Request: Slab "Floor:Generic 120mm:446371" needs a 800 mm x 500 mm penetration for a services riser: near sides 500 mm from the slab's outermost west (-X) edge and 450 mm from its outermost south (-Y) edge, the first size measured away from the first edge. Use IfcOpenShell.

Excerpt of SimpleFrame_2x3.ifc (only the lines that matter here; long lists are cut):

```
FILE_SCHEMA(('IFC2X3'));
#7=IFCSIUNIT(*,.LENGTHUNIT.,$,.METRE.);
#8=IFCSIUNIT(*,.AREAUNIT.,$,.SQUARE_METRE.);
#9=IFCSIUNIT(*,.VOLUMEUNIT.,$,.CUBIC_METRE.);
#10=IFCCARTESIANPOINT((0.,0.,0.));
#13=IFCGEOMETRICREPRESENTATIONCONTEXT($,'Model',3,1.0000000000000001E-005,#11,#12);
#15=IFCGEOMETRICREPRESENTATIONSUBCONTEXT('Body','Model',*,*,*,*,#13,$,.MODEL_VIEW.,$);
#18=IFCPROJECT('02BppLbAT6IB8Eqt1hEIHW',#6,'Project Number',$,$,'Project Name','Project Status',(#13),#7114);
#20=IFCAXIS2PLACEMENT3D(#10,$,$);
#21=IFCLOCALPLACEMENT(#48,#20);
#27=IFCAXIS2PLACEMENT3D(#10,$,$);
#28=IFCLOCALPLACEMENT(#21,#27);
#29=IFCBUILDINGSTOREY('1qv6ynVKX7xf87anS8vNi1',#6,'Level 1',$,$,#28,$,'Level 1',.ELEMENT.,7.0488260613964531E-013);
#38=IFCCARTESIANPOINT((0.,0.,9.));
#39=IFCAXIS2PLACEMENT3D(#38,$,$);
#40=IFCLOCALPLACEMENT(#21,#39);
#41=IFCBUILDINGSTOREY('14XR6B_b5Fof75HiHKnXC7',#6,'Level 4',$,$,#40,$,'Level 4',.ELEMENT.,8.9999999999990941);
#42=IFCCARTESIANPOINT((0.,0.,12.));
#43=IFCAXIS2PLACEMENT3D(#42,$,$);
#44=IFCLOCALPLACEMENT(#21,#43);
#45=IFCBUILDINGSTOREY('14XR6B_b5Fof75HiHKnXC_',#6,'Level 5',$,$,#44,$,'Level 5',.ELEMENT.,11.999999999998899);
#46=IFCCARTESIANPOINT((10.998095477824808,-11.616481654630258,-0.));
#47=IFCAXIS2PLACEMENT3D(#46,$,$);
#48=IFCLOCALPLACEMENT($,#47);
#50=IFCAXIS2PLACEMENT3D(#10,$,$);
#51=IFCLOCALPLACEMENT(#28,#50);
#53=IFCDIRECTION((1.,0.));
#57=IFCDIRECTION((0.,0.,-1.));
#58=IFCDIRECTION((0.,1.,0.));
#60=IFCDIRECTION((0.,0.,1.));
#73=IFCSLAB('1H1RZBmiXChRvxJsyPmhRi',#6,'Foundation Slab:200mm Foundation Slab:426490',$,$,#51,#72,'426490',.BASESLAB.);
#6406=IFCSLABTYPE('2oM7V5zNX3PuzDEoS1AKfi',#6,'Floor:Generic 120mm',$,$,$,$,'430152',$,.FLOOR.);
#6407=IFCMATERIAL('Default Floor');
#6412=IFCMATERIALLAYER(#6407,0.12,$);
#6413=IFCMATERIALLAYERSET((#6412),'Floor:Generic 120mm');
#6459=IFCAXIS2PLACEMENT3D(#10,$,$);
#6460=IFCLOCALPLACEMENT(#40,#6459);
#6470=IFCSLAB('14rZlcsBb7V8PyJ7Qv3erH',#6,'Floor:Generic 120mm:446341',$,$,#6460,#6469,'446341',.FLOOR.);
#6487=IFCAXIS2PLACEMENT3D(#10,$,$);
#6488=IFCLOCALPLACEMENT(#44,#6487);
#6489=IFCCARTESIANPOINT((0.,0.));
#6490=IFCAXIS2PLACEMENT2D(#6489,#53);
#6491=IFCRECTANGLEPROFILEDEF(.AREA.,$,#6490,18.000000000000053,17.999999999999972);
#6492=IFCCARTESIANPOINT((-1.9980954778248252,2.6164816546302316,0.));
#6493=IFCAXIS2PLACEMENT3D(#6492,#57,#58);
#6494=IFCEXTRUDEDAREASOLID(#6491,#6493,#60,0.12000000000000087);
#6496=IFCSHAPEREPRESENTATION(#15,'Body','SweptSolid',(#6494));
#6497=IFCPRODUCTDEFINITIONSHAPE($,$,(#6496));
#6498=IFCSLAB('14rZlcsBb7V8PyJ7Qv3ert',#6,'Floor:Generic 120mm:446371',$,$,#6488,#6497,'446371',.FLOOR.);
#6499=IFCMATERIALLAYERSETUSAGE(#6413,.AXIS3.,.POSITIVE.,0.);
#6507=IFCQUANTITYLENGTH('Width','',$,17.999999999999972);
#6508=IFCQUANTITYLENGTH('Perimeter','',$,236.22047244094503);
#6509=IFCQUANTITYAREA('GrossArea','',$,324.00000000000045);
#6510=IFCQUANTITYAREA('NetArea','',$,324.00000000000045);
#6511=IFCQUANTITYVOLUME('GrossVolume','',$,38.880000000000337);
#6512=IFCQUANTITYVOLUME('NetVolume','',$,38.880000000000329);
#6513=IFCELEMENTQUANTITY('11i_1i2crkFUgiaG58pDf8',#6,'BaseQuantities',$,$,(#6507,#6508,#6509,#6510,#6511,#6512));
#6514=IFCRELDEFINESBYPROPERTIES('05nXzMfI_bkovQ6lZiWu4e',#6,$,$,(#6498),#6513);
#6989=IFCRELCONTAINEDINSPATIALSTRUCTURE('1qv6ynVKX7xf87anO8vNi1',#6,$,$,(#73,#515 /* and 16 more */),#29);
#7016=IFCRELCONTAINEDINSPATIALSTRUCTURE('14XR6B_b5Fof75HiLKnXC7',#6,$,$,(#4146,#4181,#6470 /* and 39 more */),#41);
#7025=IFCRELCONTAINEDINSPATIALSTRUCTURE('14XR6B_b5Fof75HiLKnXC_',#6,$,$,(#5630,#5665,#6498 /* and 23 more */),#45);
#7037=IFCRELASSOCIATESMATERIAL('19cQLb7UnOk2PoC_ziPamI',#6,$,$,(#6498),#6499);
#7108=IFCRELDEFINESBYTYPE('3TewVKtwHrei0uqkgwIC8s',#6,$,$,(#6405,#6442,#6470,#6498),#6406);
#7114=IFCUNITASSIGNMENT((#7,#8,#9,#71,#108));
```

```python
import numpy as np
import ifcopenshell
import ifcopenshell.api.feature
import ifcopenshell.api.geometry
import ifcopenshell.api.pset
import ifcopenshell.api.root
import ifcopenshell.geom
import ifcopenshell.util.element
import ifcopenshell.util.placement
import ifcopenshell.util.representation
import ifcopenshell.util.shape
import ifcopenshell.util.unit

model = ifcopenshell.open("SimpleFrame_2x3.ifc")
unit_scale = ifcopenshell.util.unit.calculate_unit_scale(model)
area_scale = ifcopenshell.util.unit.calculate_unit_scale(model, "AREAUNIT")
volume_scale = ifcopenshell.util.unit.calculate_unit_scale(model, "VOLUMEUNIT")
settings = ifcopenshell.geom.settings()


def volume(element):
    """Net volume in cubic metres, openings subtracted."""
    shape = ifcopenshell.geom.create_shape(settings, element)
    return ifcopenshell.util.shape.get_volume(shape.geometry)


slab = model.by_id(6498)
before = volume(slab)

# Extent in the slab's own axes, in metres. The edges named are its -X and -Y sides.
slab_shape = ifcopenshell.geom.create_shape(settings, slab)
vertices = ifcopenshell.util.shape.get_vertices(slab_shape.geometry)
x_min, y_min, bottom = vertices.min(axis=0)
top = vertices[:, 2].max()

opening = ifcopenshell.api.root.create_entity(model, ifc_class="IfcOpeningElement", name="Services riser opening")
context = ifcopenshell.util.representation.get_context(model, "Model", "Body", "MODEL_VIEW")
width, depth = 0.8, 0.5
outline = [(0.0, 0.0), (width, 0.0), (width, depth), (0.0, depth), (0.0, 0.0)]
# Overshoot both faces by 50 mm so the cut is clean.
shape = ifcopenshell.api.geometry.add_slab_representation(
    model, context=context, depth=top - bottom + 0.1, polyline=outline
)
ifcopenshell.api.geometry.assign_representation(model, product=opening, representation=shape)

matrix = ifcopenshell.util.placement.get_local_placement(slab.ObjectPlacement)
matrix[:, 3] = matrix @ np.append(np.array([x_min + 0.5, y_min + 0.45, bottom - 0.05]) / unit_scale, 1.0)
ifcopenshell.api.geometry.edit_object_placement(model, product=opening, matrix=matrix, is_si=False)
ifcopenshell.api.feature.add_feature(model, feature=opening, element=slab)

after = volume(slab)

# Update the slab's stored quantities.
qto = model.by_id(ifcopenshell.util.element.get_pset(slab, "BaseQuantities", should_inherit=False)["id"])
ifcopenshell.api.pset.edit_qto(model, qto=qto, properties={
    "NetArea": after / (top - bottom) / area_scale,
    "NetVolume": after / volume_scale,
})

print(f"slab volume {before:.3f} -> {after:.3f} m3")

model.write("SimpleFrame_2x3-out.ifc")
```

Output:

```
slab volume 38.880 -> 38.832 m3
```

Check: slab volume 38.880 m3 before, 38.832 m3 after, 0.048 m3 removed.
